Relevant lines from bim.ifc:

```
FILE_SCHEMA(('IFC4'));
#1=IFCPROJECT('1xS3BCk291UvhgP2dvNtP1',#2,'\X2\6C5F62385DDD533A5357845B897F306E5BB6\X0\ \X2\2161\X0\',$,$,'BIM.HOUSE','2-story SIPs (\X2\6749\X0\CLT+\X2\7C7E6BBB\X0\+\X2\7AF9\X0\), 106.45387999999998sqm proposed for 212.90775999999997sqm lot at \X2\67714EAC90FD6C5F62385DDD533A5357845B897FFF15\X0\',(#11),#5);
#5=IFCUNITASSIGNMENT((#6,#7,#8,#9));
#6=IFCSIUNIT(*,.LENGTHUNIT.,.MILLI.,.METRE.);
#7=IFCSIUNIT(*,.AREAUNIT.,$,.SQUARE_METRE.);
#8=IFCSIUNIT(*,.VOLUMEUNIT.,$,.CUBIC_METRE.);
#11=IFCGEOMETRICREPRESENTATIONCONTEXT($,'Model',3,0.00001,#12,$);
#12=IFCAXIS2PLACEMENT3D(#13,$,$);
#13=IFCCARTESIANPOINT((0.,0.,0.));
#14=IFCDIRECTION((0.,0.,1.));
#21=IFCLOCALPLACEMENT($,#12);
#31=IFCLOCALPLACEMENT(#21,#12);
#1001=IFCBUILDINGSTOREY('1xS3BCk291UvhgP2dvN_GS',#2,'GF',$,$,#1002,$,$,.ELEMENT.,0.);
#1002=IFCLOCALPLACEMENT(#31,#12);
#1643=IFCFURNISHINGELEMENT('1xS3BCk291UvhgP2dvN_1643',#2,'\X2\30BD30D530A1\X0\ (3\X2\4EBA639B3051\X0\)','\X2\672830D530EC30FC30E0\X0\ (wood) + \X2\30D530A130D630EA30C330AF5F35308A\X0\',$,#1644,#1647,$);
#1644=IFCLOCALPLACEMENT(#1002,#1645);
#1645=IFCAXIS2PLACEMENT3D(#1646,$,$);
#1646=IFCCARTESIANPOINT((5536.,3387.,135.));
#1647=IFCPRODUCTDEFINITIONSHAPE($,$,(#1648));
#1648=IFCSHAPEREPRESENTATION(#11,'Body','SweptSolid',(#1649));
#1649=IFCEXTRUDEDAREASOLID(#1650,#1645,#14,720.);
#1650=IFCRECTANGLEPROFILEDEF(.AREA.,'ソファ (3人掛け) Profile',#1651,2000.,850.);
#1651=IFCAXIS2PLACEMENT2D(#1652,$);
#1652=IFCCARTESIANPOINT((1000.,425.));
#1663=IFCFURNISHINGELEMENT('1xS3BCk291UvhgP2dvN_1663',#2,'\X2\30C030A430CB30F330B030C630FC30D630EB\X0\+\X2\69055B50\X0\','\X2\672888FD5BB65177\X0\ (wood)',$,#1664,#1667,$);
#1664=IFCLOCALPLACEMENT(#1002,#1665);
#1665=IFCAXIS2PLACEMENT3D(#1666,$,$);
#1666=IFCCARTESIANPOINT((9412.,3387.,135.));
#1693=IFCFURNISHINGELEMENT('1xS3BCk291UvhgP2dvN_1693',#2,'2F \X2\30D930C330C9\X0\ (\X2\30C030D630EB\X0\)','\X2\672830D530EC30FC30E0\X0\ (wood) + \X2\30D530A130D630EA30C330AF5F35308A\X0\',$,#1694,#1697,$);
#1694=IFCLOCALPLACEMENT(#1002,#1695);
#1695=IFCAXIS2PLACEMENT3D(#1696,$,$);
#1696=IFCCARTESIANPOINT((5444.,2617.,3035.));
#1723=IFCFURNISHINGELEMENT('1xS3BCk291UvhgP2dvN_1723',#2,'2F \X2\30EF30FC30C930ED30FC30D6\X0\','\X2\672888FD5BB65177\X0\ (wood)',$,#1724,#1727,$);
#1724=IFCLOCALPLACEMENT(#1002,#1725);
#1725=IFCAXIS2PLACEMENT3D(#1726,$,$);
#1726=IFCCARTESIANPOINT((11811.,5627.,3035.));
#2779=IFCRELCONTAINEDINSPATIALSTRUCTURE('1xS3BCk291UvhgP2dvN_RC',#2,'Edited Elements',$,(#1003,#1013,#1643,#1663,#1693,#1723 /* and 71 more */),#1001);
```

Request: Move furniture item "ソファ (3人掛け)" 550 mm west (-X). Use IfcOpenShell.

```python
import ifcopenshell
import ifcopenshell.api.geometry
import ifcopenshell.util.placement
import ifcopenshell.util.unit

model = ifcopenshell.open("bim.ifc")
unit_scale = ifcopenshell.util.unit.calculate_unit_scale(model)

item = model.by_id(1643)
matrix = ifcopenshell.util.placement.get_local_placement(item.ObjectPlacement)
matrix[0, 3] -= 0.55 / unit_scale
ifcopenshell.api.geometry.edit_object_placement(model, product=item, matrix=matrix, is_si=False)

print(ifcopenshell.util.placement.get_local_placement(item.ObjectPlacement).round(3) + 0.0)

model.write("bim_v2.ifc")
```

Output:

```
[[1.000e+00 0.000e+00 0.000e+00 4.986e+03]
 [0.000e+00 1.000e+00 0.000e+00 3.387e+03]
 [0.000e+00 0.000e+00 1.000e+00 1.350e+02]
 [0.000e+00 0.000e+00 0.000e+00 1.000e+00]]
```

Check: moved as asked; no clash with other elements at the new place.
